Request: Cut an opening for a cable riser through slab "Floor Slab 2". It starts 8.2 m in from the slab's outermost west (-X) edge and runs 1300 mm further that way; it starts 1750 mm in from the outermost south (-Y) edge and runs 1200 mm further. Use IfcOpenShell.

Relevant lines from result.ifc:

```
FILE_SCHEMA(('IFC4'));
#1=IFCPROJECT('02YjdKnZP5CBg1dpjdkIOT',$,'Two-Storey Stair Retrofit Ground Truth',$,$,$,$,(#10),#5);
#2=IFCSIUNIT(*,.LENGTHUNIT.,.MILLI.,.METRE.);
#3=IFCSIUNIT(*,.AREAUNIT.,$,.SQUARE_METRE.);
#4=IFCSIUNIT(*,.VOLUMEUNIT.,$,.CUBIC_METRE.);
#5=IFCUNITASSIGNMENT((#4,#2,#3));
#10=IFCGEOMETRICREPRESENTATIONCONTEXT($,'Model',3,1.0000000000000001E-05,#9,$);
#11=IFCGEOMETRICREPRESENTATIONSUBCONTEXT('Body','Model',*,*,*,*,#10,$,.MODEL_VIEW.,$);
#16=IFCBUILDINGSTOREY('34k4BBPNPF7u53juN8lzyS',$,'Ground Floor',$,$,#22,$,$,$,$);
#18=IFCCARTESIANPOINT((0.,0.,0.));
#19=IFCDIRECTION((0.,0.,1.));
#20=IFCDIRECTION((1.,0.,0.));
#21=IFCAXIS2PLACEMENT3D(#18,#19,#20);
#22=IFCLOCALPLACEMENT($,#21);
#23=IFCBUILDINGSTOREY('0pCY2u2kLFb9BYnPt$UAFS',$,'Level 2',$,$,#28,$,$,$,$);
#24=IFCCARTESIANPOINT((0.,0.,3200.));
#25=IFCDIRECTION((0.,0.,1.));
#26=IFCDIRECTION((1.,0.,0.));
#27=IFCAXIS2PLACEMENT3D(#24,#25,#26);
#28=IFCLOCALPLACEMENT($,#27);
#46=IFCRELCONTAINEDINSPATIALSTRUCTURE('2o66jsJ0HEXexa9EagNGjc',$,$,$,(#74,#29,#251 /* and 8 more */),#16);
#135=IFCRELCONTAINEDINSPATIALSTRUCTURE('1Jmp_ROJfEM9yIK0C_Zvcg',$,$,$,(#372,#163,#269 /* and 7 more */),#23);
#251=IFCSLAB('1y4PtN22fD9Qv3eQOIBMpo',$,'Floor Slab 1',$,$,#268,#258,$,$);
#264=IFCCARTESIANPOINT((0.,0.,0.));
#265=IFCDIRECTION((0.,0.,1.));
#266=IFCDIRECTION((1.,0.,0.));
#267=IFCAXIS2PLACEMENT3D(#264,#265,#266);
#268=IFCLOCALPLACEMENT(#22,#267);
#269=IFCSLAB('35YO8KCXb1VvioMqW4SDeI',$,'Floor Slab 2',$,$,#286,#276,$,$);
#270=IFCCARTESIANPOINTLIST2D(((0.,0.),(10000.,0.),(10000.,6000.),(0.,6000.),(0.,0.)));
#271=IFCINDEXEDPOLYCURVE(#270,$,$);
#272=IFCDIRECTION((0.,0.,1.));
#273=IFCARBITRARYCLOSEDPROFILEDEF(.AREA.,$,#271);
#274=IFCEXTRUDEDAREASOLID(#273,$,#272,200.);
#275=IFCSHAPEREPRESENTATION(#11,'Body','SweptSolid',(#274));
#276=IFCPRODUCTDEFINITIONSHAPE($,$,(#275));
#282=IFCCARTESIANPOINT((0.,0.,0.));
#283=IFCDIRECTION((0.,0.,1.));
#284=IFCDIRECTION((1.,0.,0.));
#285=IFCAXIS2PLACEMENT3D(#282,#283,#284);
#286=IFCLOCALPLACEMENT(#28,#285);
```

```python
import numpy as np
import ifcopenshell
import ifcopenshell.api.feature
import ifcopenshell.api.geometry
import ifcopenshell.api.root
import ifcopenshell.geom
import ifcopenshell.util.placement
import ifcopenshell.util.representation
import ifcopenshell.util.shape
import ifcopenshell.util.unit

model = ifcopenshell.open("result.ifc")
unit_scale = ifcopenshell.util.unit.calculate_unit_scale(model)
settings = ifcopenshell.geom.settings()


def volume(element):
    """Net volume in cubic metres, openings subtracted."""
    shape = ifcopenshell.geom.create_shape(settings, element)
    return ifcopenshell.util.shape.get_volume(shape.geometry)


slab = model.by_guid("35YO8KCXb1VvioMqW4SDeI")
before = volume(slab)

# Extent in the slab's own axes, in metres. The edges named are its -X and -Y sides.
slab_shape = ifcopenshell.geom.create_shape(settings, slab)
vertices = ifcopenshell.util.shape.get_vertices(slab_shape.geometry)
x_min, y_min, bottom = vertices.min(axis=0)
top = vertices[:, 2].max()

opening = ifcopenshell.api.root.create_entity(model, ifc_class="IfcOpeningElement", name="Cable riser opening", predefined_type="OPENING")
context = ifcopenshell.util.representation.get_context(model, "Model", "Body", "MODEL_VIEW")
width, depth = 1.3, 1.2
outline = [(0.0, 0.0), (width, 0.0), (width, depth), (0.0, depth), (0.0, 0.0)]
# Overshoot both faces by 50 mm so the cut is clean.
shape = ifcopenshell.api.geometry.add_slab_representation(
    model, context=context, depth=top - bottom + 0.1, polyline=outline
)
ifcopenshell.api.geometry.assign_representation(model, product=opening, representation=shape)

matrix = ifcopenshell.util.placement.get_local_placement(slab.ObjectPlacement)
matrix[:, 3] = matrix @ np.append(np.array([x_min + 8.2, y_min + 1.75, bottom - 0.05]) / unit_scale, 1.0)
ifcopenshell.api.geometry.edit_object_placement(model, product=opening, matrix=matrix, is_si=False)
ifcopenshell.api.feature.add_feature(model, feature=opening, element=slab)

after = volume(slab)

print(f"slab volume {before:.3f} -> {after:.3f} m3")

model.write("result_updated.ifc")
```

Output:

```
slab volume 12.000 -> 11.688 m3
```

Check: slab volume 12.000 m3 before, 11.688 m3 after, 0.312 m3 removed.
